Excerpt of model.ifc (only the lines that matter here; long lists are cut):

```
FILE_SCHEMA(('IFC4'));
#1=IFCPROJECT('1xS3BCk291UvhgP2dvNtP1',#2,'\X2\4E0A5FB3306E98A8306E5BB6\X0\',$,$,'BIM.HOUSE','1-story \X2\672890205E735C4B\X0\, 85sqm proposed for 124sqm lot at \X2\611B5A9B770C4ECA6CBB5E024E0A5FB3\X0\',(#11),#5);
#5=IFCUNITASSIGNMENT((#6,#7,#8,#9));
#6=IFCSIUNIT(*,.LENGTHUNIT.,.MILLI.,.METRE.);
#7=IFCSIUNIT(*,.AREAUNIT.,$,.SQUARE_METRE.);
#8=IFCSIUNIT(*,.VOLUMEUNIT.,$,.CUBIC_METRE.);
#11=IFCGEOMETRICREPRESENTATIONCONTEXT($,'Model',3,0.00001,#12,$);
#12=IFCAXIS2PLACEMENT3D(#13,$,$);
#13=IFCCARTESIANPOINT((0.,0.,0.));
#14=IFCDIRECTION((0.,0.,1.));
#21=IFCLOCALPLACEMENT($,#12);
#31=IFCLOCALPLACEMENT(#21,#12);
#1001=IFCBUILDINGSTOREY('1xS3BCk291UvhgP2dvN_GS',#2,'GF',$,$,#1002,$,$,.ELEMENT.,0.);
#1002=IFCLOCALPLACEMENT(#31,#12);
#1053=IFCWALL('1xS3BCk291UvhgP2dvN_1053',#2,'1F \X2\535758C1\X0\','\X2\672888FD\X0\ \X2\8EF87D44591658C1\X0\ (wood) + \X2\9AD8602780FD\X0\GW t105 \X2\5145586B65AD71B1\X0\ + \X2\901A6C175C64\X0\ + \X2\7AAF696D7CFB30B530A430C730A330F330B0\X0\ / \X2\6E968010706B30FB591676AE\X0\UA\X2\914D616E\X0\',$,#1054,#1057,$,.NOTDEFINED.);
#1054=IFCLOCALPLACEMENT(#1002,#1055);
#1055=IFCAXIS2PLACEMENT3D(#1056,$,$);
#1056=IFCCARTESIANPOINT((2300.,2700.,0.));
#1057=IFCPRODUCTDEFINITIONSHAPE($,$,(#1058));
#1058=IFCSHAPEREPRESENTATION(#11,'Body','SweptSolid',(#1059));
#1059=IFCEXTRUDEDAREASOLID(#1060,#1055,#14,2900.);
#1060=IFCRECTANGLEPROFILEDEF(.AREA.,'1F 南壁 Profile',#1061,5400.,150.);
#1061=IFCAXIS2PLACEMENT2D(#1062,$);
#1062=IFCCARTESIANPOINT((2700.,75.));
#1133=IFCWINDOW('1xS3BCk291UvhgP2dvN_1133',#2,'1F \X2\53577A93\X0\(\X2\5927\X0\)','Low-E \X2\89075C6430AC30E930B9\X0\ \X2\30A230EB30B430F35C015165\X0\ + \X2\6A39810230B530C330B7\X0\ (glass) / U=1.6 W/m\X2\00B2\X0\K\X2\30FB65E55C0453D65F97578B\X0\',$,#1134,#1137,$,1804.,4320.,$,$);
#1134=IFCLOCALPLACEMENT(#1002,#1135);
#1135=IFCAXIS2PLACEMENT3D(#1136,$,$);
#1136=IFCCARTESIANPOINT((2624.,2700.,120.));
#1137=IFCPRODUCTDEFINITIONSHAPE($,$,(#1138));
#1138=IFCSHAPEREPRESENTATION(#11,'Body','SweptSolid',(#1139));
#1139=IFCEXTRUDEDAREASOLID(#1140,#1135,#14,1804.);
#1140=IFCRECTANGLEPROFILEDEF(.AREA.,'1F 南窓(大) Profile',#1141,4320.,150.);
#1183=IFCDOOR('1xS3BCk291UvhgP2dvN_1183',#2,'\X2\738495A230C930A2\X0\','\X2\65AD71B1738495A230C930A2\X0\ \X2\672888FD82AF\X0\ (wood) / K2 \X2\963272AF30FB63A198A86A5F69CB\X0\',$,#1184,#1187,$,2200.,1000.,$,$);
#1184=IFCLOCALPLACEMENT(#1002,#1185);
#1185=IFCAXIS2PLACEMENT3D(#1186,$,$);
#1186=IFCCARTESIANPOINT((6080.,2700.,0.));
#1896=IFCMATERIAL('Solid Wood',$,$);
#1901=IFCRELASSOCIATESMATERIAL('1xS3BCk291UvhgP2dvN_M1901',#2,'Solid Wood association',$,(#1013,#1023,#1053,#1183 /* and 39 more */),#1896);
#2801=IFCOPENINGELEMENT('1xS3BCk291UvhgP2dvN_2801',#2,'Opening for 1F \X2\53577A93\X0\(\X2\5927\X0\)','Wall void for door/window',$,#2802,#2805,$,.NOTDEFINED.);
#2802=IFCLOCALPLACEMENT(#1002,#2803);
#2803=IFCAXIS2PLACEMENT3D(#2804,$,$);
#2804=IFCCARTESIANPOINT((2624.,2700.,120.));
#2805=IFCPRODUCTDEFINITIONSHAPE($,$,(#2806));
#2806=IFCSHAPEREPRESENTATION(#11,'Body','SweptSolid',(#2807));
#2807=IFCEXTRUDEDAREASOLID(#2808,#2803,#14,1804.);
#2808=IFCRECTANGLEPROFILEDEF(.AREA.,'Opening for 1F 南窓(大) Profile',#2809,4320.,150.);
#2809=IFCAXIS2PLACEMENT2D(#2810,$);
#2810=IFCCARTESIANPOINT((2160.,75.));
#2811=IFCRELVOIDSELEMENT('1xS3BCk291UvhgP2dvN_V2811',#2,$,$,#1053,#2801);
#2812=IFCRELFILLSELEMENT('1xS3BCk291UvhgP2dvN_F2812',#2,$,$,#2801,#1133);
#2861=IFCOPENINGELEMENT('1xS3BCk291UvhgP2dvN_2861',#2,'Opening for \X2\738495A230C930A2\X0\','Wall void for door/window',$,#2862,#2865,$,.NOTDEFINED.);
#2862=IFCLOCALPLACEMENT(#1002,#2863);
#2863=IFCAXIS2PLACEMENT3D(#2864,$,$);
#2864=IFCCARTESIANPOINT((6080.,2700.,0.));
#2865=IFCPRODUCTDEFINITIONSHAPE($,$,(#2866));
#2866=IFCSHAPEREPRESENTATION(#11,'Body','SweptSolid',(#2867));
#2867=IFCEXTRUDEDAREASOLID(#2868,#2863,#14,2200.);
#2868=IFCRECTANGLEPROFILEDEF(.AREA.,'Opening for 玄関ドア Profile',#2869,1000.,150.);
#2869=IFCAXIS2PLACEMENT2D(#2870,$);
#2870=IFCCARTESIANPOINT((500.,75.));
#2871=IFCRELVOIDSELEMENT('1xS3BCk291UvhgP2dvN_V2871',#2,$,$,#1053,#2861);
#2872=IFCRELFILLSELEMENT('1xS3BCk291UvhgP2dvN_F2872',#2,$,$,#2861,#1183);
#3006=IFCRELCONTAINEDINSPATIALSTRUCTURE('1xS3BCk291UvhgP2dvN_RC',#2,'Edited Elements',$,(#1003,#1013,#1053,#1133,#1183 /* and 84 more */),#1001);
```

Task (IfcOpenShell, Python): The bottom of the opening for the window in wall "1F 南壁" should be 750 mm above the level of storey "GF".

```python
import numpy as np
import ifcopenshell
import ifcopenshell.api.geometry
import ifcopenshell.geom
import ifcopenshell.util.element
import ifcopenshell.util.placement
import ifcopenshell.util.shape
import ifcopenshell.util.unit

model = ifcopenshell.open("model.ifc")
unit_scale = ifcopenshell.util.unit.calculate_unit_scale(model)

window = model.by_guid("1xS3BCk291UvhgP2dvN_1133")
opening = window.FillsVoids[0].RelatingOpeningElement
storey = ifcopenshell.util.element.get_container(window, ifc_class="IfcBuildingStorey")
level = ifcopenshell.util.placement.get_local_placement(storey.ObjectPlacement)[2, 3]

# The opening's origin need not be at the sill, so measure its lowest point.
shape = ifcopenshell.geom.create_shape(ifcopenshell.geom.settings(), opening)
bottom = ifcopenshell.util.shape.get_shape_bottom_elevation(shape, shape.geometry) / unit_scale
dz = level + 0.75 / unit_scale - bottom

shift = np.array([0.0, 0.0, dz])
# The window is not placed relative to its opening, so move both.
for product in (opening, window):
    matrix = ifcopenshell.util.placement.get_local_placement(product.ObjectPlacement)
    matrix[:3, 3] += shift
    ifcopenshell.api.geometry.edit_object_placement(model, product=product, matrix=matrix, is_si=False)

print(f"moved by {dz * unit_scale:+.3f} m")

model.write("model_v2.ifc")
```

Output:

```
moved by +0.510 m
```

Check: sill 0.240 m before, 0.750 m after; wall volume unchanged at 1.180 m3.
